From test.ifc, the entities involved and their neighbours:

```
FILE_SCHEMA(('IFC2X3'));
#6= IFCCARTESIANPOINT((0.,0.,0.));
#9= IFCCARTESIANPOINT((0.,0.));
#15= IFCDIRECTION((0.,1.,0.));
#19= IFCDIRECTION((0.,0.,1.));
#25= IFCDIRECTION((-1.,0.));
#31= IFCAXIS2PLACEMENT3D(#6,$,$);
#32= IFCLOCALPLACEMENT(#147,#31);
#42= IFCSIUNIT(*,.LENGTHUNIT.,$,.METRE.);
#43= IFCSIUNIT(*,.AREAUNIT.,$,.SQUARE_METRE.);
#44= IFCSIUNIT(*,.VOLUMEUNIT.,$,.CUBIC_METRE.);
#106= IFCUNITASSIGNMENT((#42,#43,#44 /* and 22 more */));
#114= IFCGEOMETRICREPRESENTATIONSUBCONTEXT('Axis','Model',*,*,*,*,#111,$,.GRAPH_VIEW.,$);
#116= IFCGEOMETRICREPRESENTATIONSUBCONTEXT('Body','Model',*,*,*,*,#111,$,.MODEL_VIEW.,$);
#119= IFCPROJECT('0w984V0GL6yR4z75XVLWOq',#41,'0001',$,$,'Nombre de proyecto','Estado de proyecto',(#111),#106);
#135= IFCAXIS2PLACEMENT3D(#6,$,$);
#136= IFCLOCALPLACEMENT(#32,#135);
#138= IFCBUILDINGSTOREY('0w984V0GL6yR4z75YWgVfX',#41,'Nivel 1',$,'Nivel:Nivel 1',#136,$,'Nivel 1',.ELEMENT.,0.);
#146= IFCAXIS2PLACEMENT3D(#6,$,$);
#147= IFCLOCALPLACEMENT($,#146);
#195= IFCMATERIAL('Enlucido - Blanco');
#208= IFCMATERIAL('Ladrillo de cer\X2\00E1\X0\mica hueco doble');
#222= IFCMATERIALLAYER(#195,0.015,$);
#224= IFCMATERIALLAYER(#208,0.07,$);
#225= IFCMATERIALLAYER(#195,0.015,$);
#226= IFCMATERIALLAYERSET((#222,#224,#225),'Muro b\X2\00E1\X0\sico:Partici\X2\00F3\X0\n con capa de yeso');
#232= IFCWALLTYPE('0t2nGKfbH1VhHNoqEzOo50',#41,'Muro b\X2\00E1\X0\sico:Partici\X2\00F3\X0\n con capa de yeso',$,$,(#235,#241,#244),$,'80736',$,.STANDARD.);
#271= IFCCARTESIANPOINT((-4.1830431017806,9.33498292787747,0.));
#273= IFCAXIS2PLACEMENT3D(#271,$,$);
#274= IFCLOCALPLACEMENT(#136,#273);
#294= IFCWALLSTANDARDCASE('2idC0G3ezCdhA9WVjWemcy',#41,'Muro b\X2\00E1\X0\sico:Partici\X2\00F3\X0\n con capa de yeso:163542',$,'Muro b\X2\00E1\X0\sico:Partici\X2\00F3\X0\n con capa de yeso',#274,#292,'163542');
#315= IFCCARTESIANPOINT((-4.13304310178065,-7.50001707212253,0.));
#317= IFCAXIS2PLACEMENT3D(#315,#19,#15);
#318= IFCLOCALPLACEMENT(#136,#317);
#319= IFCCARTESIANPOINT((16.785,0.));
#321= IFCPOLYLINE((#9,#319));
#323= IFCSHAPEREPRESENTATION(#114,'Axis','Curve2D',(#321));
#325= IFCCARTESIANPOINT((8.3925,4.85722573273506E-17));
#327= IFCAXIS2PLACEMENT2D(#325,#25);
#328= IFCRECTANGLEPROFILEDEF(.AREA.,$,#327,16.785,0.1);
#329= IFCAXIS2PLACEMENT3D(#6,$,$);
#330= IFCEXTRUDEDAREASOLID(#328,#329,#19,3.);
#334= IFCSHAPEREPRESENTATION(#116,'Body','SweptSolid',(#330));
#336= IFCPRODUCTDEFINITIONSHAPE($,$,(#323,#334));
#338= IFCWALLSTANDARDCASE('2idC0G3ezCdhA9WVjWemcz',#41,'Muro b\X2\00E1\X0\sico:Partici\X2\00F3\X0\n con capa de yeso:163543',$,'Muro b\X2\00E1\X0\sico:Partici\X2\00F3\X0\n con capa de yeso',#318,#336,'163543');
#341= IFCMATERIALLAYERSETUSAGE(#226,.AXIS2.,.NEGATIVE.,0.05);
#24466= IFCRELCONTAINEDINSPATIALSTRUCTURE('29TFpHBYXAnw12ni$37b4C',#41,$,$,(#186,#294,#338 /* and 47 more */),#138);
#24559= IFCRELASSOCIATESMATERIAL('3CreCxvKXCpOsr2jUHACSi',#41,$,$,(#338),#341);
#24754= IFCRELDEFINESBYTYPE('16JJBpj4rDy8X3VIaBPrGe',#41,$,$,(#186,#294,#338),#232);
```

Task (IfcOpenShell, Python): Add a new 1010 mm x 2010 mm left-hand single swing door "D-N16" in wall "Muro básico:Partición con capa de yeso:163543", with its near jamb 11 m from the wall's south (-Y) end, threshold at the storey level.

```python
import numpy as np
import ifcopenshell
import ifcopenshell.api.feature
import ifcopenshell.api.geometry
import ifcopenshell.api.root
import ifcopenshell.api.spatial
import ifcopenshell.api.type
import ifcopenshell.geom
import ifcopenshell.util.element
import ifcopenshell.util.placement
import ifcopenshell.util.representation
import ifcopenshell.util.shape
import ifcopenshell.util.unit

model = ifcopenshell.open("test.ifc")
unit_scale = ifcopenshell.util.unit.calculate_unit_scale(model)
settings = ifcopenshell.geom.settings()


def volume(element):
    """Net volume in cubic metres, openings subtracted."""
    shape = ifcopenshell.geom.create_shape(settings, element)
    return ifcopenshell.util.shape.get_volume(shape.geometry)


wall = model.by_guid("2idC0G3ezCdhA9WVjWemcz")
storey = ifcopenshell.util.element.get_container(wall, ifc_class="IfcBuildingStorey")
context = ifcopenshell.util.representation.get_context(model, "Model", "Body", "MODEL_VIEW")
before = volume(wall)

width, height, from_end, sill = 1.01, 2.01, 11, 0.0  # metres

# The wall runs along its own X axis, and the end named is its -X end.
wall_shape = ifcopenshell.geom.create_shape(settings, wall)
x, y, z = ifcopenshell.util.shape.get_vertices(wall_shape.geometry).T
start = x.min() + from_end
face, thickness = float(y.min()), float(y.max() - y.min())
wall_matrix = ifcopenshell.util.placement.get_local_placement(wall.ObjectPlacement)
level = ifcopenshell.util.placement.get_local_placement(storey.ObjectPlacement)[2, 3]


def in_wall(x, y):
    """Placement at x, y metres in the wall's axes, at sill height."""
    matrix = wall_matrix.copy()
    matrix[:, 3] = wall_matrix @ np.array([x / unit_scale, y / unit_scale, 0.0, 1.0])
    matrix[2, 3] = level + sill / unit_scale
    return matrix


# Opening: a box that overshoots both wall faces by 50 mm.
opening = ifcopenshell.api.root.create_entity(model, ifc_class="IfcOpeningElement")
box = ifcopenshell.api.geometry.add_wall_representation(
    model, context=context, length=width, height=height, thickness=thickness + 0.1
)
ifcopenshell.api.geometry.assign_representation(model, product=opening, representation=box)
ifcopenshell.api.geometry.edit_object_placement(model, product=opening, matrix=in_wall(start, face - 0.05), is_si=False)
ifcopenshell.api.feature.add_feature(model, feature=opening, element=wall)

door = ifcopenshell.api.root.create_entity(model, ifc_class="IfcDoor", name="D-N16")
door.OverallWidth, door.OverallHeight = width / unit_scale, height / unit_scale
body = ifcopenshell.api.geometry.add_door_representation(
    model,
    context=context,
    overall_width=door.OverallWidth,
    overall_height=door.OverallHeight,
    operation_type="SINGLE_SWING_LEFT",
    lining_properties={"LiningDepth": thickness / unit_scale, "ThresholdDepth": thickness / unit_scale},
)
ifcopenshell.api.geometry.assign_representation(model, product=door, representation=body)
ifcopenshell.api.spatial.assign_container(model, products=[door], relating_structure=storey)
fills = ifcopenshell.api.feature.add_filling(model, opening=opening, element=door)
fills.OwnerHistory = door.OwnerHistory  # required in IFC2X3

# IFC2X3 keeps the operation on the door style.
style = ifcopenshell.api.root.create_entity(model, ifc_class="IfcDoorStyle", name="D-N16")
style.OperationType, style.ConstructionType = "SINGLE_SWING_LEFT", "NOTDEFINED"
style.ParameterTakesPrecedence = style.Sizeable = False
ifcopenshell.api.type.assign_type(model, related_objects=[door], relating_type=style)

# The lining spans the wall, so the door starts at the wall face.
ifcopenshell.api.geometry.edit_object_placement(model, product=door, matrix=in_wall(start, face), is_si=False)

after = volume(wall)

print(f"wall volume {before:.3f} -> {after:.3f} m3")

model.write("test_rev.ifc")
```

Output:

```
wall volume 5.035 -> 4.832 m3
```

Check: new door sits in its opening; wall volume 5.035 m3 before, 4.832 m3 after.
